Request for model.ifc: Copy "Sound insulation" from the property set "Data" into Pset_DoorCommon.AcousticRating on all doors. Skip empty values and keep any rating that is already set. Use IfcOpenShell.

First a look at what the model holds.

```python
import ifcopenshell
import ifcopenshell.util.element

model = ifcopenshell.open("model.ifc")
print(model.schema)
doors = model.by_type("IfcDoor")
print(len(doors), "doors")
for e in doors[:8]:
    source = ifcopenshell.util.element.get_pset(e, "Data", "Sound insulation")
    target = ifcopenshell.util.element.get_pset(e, "Pset_DoorCommon", "AcousticRating")
    print(e.id(), repr(source), repr(target), sep=" | ")
```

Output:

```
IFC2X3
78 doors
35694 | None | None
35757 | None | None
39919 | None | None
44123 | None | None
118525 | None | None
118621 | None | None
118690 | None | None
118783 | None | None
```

```python
import ifcopenshell
import ifcopenshell.api.pset
import ifcopenshell.util.element

model = ifcopenshell.open("model.ifc")

count = 0
for e in model.by_type("IfcDoor"):
    value = ifcopenshell.util.element.get_pset(e, "Data", "Sound insulation")
    current = ifcopenshell.util.element.get_pset(e, "Pset_DoorCommon", "AcousticRating")
    if not value or not value.strip() or current:
        continue
    # add_pset returns the element's existing set when there is one.
    pset = ifcopenshell.api.pset.add_pset(model, product=e, name="Pset_DoorCommon")
    ifcopenshell.api.pset.edit_pset(model, pset=pset, properties={"AcousticRating": value})
    count += 1

print(count, "doors updated")

model.write("model_v2.ifc")
```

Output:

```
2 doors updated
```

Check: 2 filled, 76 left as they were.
